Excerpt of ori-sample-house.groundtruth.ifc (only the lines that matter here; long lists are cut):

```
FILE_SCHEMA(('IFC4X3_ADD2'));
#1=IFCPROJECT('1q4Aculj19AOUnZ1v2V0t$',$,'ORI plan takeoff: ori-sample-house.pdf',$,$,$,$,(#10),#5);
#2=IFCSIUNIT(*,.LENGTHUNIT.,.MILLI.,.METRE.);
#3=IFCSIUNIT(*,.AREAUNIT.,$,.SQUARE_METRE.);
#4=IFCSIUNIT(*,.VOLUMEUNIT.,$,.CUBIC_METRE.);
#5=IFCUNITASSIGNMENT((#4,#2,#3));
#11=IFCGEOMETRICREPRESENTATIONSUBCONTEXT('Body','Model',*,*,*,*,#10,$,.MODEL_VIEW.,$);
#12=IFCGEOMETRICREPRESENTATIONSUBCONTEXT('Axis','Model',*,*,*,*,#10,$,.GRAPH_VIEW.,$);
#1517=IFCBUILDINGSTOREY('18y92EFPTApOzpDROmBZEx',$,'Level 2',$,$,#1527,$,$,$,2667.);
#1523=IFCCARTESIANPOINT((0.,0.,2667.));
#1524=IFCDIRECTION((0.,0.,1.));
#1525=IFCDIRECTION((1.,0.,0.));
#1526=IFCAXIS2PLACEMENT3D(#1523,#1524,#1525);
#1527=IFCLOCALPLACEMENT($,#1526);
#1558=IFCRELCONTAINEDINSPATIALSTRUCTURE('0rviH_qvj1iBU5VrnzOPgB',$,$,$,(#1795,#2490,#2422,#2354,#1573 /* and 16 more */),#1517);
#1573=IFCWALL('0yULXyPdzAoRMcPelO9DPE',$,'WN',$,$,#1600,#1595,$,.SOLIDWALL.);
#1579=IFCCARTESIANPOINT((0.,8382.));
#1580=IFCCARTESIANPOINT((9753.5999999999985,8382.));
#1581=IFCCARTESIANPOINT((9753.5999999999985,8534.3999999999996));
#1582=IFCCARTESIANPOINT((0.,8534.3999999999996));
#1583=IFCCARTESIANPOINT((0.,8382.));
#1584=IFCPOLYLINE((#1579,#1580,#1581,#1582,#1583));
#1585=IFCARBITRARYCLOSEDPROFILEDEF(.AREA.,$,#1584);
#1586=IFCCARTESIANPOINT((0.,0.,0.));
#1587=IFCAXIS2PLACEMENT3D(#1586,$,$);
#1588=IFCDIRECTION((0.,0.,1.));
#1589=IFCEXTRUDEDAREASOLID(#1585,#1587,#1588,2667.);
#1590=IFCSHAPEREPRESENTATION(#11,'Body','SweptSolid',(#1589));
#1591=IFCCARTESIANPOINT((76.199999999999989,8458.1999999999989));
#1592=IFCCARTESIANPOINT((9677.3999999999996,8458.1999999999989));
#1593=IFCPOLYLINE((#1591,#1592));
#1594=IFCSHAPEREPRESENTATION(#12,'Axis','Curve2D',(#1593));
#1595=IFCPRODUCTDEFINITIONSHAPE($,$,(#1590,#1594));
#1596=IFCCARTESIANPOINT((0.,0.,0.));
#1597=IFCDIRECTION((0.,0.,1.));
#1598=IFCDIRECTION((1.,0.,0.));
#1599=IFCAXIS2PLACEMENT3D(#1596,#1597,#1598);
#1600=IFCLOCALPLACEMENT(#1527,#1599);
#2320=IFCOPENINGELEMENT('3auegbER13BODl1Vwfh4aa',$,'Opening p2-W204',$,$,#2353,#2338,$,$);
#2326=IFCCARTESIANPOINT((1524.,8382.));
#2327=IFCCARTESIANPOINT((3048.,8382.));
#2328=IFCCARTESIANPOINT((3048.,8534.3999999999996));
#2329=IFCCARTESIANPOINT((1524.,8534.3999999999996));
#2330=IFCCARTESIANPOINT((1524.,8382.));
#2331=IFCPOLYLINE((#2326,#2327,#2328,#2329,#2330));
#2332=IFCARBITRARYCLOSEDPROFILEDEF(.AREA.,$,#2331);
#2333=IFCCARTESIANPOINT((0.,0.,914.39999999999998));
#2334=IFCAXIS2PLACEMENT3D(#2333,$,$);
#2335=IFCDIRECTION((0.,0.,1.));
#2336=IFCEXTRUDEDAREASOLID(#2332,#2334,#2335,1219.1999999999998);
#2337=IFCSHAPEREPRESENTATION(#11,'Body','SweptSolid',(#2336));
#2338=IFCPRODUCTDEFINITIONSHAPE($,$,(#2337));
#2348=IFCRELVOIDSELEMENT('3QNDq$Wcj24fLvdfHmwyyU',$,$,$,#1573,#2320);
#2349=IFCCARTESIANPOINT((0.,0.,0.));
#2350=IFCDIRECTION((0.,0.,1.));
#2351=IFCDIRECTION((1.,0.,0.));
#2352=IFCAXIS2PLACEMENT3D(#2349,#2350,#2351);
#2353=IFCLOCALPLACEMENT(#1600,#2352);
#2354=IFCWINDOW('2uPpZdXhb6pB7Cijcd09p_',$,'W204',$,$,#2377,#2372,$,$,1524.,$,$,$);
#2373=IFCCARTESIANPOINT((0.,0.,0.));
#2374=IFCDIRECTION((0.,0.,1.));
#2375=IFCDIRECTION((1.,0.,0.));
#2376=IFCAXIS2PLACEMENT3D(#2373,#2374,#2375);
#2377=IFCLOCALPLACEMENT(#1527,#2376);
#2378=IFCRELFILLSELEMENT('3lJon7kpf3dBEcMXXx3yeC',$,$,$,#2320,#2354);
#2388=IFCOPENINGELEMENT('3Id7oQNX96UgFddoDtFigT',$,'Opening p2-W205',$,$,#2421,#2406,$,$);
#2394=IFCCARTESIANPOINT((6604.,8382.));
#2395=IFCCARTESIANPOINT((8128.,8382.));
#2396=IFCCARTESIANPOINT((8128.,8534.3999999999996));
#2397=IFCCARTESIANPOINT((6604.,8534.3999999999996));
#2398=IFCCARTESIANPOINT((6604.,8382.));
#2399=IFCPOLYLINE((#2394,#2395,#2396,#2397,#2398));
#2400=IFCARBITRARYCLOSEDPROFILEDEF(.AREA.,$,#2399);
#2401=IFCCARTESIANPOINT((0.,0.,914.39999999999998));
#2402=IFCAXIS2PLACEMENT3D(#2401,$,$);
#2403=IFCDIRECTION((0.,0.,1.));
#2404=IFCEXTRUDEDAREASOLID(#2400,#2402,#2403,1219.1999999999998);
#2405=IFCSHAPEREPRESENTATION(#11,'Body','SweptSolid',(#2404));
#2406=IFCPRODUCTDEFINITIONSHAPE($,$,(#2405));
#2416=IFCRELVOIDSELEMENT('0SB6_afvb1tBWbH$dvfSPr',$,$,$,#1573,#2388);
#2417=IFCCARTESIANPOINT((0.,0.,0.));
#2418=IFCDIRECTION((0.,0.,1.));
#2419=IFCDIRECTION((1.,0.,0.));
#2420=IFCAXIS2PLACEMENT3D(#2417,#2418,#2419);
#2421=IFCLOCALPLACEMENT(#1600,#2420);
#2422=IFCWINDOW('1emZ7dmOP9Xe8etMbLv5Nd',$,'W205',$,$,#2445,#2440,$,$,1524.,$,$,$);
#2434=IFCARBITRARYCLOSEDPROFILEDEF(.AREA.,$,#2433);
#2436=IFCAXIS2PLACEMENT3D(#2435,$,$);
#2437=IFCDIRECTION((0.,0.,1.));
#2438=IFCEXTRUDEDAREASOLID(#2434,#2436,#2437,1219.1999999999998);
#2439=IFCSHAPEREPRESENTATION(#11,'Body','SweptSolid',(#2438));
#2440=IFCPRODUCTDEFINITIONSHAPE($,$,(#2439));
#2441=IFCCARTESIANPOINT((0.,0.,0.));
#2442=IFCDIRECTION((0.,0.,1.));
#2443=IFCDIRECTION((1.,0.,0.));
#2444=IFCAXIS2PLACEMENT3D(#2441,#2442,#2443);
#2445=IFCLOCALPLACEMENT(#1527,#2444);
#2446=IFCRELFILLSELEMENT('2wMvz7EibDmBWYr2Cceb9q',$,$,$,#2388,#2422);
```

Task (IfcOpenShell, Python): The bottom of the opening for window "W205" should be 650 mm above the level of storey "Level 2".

```python
import numpy as np
import ifcopenshell
import ifcopenshell.api.geometry
import ifcopenshell.geom
import ifcopenshell.util.element
import ifcopenshell.util.placement
import ifcopenshell.util.shape
import ifcopenshell.util.unit

model = ifcopenshell.open("ori-sample-house.groundtruth.ifc")
unit_scale = ifcopenshell.util.unit.calculate_unit_scale(model)

window = model.by_id(2422)
opening = window.FillsVoids[0].RelatingOpeningElement
storey = ifcopenshell.util.element.get_container(window, ifc_class="IfcBuildingStorey")
level = ifcopenshell.util.placement.get_local_placement(storey.ObjectPlacement)[2, 3]

# The opening's origin need not be at the sill, so measure its lowest point.
shape = ifcopenshell.geom.create_shape(ifcopenshell.geom.settings(), opening)
bottom = ifcopenshell.util.shape.get_shape_bottom_elevation(shape, shape.geometry) / unit_scale
dz = level + 0.65 / unit_scale - bottom

shift = np.array([0.0, 0.0, dz])
# The window is not placed relative to its opening, so move both.
for product in (opening, window):
    matrix = ifcopenshell.util.placement.get_local_placement(product.ObjectPlacement)
    matrix[:3, 3] += shift
    ifcopenshell.api.geometry.edit_object_placement(model, product=product, matrix=matrix, is_si=False)

print(f"moved by {dz * unit_scale:+.3f} m")

model.write("ori-sample-house.groundtruth_updated.ifc")
```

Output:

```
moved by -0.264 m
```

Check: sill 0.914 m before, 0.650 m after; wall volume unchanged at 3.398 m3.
